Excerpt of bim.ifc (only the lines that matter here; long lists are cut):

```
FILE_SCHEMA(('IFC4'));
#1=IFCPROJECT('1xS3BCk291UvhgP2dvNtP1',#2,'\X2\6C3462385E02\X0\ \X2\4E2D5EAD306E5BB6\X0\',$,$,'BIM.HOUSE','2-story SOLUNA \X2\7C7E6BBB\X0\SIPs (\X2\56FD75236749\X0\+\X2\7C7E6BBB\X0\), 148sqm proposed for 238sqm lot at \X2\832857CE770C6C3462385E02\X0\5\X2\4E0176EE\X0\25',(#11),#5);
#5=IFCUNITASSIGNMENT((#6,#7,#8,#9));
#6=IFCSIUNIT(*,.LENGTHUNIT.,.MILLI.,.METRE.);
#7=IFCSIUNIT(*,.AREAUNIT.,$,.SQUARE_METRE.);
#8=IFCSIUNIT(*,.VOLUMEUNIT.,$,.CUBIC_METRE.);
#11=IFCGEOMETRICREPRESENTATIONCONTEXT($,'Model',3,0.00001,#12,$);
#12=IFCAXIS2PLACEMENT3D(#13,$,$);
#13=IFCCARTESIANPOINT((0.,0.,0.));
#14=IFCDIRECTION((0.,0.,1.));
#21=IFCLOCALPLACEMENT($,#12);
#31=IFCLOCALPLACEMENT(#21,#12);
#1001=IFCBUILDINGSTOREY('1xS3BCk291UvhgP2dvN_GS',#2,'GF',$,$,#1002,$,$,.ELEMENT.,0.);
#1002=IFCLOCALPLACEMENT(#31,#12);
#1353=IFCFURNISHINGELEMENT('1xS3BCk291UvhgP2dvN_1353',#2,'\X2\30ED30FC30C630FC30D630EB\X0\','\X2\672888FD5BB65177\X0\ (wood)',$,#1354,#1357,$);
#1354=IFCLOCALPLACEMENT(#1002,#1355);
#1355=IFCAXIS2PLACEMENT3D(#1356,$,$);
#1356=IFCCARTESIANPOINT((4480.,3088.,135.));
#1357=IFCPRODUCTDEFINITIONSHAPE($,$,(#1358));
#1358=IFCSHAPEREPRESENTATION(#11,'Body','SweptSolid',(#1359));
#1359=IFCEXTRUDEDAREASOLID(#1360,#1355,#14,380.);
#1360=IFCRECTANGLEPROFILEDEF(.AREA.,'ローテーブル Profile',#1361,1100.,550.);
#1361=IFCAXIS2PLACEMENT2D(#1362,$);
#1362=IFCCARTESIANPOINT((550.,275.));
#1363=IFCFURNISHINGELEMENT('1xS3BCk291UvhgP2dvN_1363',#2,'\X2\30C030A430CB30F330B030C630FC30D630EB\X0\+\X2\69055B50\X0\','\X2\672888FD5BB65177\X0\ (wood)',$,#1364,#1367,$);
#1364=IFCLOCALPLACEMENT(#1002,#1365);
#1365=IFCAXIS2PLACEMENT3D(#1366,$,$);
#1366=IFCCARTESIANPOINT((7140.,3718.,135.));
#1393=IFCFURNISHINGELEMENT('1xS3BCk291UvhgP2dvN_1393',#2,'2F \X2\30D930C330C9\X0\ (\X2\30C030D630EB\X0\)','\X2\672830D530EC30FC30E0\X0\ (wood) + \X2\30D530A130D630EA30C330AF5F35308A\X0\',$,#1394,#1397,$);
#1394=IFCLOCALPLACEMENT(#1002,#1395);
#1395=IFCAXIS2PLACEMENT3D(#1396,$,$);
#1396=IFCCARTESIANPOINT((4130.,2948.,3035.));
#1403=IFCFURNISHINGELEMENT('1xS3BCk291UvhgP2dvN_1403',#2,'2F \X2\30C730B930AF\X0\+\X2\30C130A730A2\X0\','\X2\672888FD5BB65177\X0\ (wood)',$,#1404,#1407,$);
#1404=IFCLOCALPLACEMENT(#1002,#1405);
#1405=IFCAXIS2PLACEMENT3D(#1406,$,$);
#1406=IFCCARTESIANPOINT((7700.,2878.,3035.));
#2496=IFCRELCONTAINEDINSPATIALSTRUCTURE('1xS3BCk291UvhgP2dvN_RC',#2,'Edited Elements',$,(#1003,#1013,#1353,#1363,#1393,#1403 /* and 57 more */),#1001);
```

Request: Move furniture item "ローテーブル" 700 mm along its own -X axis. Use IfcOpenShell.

```python
import ifcopenshell
import ifcopenshell.api.geometry
import ifcopenshell.util.placement
import ifcopenshell.util.unit

model = ifcopenshell.open("bim.ifc")
unit_scale = ifcopenshell.util.unit.calculate_unit_scale(model)

item = model.by_guid("1xS3BCk291UvhgP2dvN_1353")
matrix = ifcopenshell.util.placement.get_local_placement(item.ObjectPlacement)
matrix[:3, 3] -= matrix[:3, 0] * 0.7 / unit_scale
ifcopenshell.api.geometry.edit_object_placement(model, product=item, matrix=matrix, is_si=False)

print(ifcopenshell.util.placement.get_local_placement(item.ObjectPlacement).round(3) + 0.0)

model.write("bim-out.ifc")
```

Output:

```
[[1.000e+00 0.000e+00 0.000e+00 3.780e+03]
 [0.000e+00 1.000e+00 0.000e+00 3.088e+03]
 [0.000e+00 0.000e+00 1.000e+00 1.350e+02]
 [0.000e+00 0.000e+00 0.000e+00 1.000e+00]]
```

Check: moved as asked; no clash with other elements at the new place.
